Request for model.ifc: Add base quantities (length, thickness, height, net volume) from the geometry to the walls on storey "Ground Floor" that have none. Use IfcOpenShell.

First a look at what the model holds.

```python
import ifcopenshell
import ifcopenshell.util.element
import ifcopenshell.util.unit

model = ifcopenshell.open("model.ifc")
print(model.schema)
for unit_type in ("LENGTHUNIT", "AREAUNIT", "VOLUMEUNIT"):
    print(unit_type, ifcopenshell.util.unit.calculate_unit_scale(model, unit_type))
storey = next(s for s in model.by_type("IfcBuildingStorey") if s.Name == "Ground Floor")
walls = [e for e in ifcopenshell.util.element.get_decomposition(storey) if e.is_a("IfcWall")]
for e in sorted(walls, key=lambda e: e.id()):
    print(e.id(), e.is_a(), e.Name, list(ifcopenshell.util.element.get_psets(e, qtos_only=True)), sep=" | ")
```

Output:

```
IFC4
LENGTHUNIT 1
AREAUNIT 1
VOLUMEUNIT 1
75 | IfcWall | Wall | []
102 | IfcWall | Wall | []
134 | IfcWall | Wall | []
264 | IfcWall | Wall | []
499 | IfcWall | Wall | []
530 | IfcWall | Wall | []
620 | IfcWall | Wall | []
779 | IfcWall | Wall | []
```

```python
import ifcopenshell
import ifcopenshell.api.pset
import ifcopenshell.geom
import ifcopenshell.util.element
import ifcopenshell.util.shape
import ifcopenshell.util.unit

model = ifcopenshell.open("model.ifc")
unit_scale = ifcopenshell.util.unit.calculate_unit_scale(model)
volume_scale = ifcopenshell.util.unit.calculate_unit_scale(model, "VOLUMEUNIT")
settings = ifcopenshell.geom.settings()

storey = next(s for s in model.by_type("IfcBuildingStorey") if s.Name == "Ground Floor")
walls = [e for e in ifcopenshell.util.element.get_decomposition(storey) if e.is_a("IfcWall")]

for e in sorted(walls, key=lambda e: e.id()):
    if ifcopenshell.util.element.get_psets(e, qtos_only=True, should_inherit=False):
        continue
    # Geometry comes back in metres, in the element's own axes.
    shape = ifcopenshell.geom.create_shape(settings, e)
    values = {
        "Length": ifcopenshell.util.shape.get_x(shape.geometry) / unit_scale,
        "Width": ifcopenshell.util.shape.get_y(shape.geometry) / unit_scale,
        "Height": ifcopenshell.util.shape.get_z(shape.geometry) / unit_scale,
        "NetVolume": ifcopenshell.util.shape.get_volume(shape.geometry) / volume_scale,
    }
    qto = ifcopenshell.api.pset.add_qto(model, product=e, name="Qto_WallBaseQuantities")
    ifcopenshell.api.pset.edit_qto(model, qto=qto, properties=values)
    print(e.id(), {k: round(v, 3) for k, v in values.items()})

model.write("model_v2.ifc")
```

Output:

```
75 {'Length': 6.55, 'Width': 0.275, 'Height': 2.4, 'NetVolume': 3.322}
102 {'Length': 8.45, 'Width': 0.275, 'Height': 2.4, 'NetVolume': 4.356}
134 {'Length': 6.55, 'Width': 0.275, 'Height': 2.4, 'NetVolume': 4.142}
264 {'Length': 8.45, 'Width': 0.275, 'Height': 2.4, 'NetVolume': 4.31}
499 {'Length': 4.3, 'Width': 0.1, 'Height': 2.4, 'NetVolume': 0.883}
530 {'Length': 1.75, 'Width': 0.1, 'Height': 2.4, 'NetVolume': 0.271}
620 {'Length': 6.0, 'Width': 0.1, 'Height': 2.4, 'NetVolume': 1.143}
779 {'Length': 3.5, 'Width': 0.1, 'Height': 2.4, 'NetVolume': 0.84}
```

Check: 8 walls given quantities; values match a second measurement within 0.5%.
